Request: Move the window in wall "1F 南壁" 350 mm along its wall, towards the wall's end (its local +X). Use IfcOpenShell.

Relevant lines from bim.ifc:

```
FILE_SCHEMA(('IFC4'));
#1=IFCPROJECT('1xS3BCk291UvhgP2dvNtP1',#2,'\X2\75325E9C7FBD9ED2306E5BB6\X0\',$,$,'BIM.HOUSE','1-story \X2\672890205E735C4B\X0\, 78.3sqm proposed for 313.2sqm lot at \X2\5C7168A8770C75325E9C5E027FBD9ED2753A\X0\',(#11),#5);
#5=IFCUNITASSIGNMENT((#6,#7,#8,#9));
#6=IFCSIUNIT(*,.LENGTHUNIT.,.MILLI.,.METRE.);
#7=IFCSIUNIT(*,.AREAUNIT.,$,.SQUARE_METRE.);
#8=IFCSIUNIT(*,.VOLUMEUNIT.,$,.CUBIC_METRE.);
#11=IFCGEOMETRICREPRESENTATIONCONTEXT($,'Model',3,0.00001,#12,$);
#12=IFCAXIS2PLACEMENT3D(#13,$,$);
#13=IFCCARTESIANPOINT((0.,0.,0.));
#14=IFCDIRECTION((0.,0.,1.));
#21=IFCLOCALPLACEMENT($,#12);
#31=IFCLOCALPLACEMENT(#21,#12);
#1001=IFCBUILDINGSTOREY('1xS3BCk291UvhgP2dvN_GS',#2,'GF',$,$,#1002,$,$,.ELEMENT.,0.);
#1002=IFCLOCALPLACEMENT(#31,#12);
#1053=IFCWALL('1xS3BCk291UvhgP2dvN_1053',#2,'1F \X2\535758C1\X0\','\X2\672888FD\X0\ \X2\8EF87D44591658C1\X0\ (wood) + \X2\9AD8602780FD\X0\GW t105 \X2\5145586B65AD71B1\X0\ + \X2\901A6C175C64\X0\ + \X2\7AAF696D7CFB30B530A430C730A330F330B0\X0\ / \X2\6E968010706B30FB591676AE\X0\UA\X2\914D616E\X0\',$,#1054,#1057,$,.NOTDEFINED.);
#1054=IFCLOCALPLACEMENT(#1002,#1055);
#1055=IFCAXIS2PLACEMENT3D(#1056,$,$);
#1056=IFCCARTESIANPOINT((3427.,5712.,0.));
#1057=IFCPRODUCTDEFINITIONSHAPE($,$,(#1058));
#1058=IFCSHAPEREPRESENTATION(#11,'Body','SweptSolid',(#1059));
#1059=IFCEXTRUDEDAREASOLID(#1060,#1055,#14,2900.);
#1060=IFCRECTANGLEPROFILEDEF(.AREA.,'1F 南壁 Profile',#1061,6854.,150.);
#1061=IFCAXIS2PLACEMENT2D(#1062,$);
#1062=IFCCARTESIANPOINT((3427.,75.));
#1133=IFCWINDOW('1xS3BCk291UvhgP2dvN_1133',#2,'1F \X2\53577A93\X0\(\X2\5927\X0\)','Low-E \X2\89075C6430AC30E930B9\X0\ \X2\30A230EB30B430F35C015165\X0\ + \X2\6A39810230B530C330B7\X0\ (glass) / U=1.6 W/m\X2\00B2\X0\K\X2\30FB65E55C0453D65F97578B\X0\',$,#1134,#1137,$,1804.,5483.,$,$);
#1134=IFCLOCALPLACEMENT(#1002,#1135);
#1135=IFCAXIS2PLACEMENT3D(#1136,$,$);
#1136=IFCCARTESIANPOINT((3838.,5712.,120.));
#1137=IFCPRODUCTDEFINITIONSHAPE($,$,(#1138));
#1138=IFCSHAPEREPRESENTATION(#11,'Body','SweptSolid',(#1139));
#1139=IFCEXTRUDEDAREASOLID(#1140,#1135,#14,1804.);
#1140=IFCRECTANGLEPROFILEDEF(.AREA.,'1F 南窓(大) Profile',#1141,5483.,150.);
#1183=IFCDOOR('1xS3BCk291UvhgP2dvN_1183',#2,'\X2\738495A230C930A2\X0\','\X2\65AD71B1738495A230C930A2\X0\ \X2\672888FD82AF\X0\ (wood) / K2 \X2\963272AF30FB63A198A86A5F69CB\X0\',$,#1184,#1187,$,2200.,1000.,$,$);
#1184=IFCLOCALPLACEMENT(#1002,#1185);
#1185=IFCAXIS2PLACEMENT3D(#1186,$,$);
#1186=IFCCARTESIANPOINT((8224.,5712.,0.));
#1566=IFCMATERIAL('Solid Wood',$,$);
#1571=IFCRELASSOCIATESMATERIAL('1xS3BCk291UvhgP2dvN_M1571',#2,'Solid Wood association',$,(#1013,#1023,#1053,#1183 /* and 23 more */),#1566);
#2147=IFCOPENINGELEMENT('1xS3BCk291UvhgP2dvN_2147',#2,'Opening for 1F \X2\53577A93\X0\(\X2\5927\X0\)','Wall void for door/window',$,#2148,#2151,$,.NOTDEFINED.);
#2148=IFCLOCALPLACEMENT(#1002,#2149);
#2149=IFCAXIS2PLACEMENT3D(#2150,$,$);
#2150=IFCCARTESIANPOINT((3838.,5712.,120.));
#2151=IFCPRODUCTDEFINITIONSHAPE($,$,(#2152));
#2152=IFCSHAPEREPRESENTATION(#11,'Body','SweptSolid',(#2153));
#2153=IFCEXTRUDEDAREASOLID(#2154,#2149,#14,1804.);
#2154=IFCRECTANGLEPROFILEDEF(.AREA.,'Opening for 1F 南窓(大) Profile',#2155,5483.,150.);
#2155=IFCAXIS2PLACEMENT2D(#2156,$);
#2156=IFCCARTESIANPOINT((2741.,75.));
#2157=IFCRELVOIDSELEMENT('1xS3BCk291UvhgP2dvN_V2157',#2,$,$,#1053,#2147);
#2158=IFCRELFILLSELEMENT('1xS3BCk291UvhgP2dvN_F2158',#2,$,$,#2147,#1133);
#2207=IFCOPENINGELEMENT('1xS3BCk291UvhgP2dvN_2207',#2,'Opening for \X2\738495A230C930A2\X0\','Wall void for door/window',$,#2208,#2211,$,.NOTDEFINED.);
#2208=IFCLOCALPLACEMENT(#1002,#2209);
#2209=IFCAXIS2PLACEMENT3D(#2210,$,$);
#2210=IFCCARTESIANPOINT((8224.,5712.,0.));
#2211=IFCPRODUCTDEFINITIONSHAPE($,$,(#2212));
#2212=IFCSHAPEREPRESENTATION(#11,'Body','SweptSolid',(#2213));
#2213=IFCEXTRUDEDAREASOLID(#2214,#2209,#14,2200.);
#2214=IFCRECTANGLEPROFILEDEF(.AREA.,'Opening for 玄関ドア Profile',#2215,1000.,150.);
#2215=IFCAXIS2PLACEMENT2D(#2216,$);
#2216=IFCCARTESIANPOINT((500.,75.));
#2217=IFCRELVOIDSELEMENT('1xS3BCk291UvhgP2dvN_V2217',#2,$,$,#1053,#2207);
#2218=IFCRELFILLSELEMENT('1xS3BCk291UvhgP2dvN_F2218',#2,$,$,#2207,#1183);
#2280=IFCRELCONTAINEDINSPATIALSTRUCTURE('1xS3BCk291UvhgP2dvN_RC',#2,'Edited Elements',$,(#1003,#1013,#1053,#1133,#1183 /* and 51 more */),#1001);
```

```python
import ifcopenshell
import ifcopenshell.api.geometry
import ifcopenshell.util.placement
import ifcopenshell.util.unit

model = ifcopenshell.open("bim.ifc")
unit_scale = ifcopenshell.util.unit.calculate_unit_scale(model)

window = model.by_id(1133)
opening = window.FillsVoids[0].RelatingOpeningElement
wall = opening.VoidsElements[0].RelatingBuildingElement

wall_matrix = ifcopenshell.util.placement.get_local_placement(wall.ObjectPlacement)
shift = wall_matrix[:3, 0] * 0.35 / unit_scale
before = ifcopenshell.util.placement.get_local_placement(window.ObjectPlacement)[:3, 3].copy()

# The window is not placed relative to its opening, so move both.
for product in (opening, window):
    matrix = ifcopenshell.util.placement.get_local_placement(product.ObjectPlacement)
    matrix[:3, 3] += shift
    ifcopenshell.api.geometry.edit_object_placement(model, product=product, matrix=matrix, is_si=False)

after = ifcopenshell.util.placement.get_local_placement(window.ObjectPlacement)[:3, 3]
print("window moved by", (after - before).round(3) + 0.0)

model.write("bim_rev.ifc")
```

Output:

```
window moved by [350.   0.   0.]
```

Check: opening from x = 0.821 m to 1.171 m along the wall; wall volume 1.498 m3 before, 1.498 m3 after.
